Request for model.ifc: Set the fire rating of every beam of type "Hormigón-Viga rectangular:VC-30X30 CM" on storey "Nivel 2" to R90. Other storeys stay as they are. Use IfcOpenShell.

First a look at what the model holds.

```python
import ifcopenshell
import ifcopenshell.util.element

model = ifcopenshell.open("model.ifc")
print(model.schema)
storey = next(s for s in model.by_type("IfcBuildingStorey") if s.Name == "Nivel 2")
beams = [e for e in ifcopenshell.util.element.get_decomposition(storey) if e.is_a("IfcBeam")]
seen = {}
for e in beams:
    element_type = ifcopenshell.util.element.get_type(e)
    key = (element_type.Name if element_type != e and element_type else None, ifcopenshell.util.element.get_pset(e, "Pset_BeamCommon", "FireRating"))
    seen[key] = seen.get(key, 0) + 1
for (name, value), count in sorted(seen.items(), key=str):
    print(count, "x", name, "|", value)
```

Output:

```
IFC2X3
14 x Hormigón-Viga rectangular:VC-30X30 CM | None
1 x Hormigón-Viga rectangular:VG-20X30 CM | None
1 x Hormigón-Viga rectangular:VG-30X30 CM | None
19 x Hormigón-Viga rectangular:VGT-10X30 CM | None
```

```python
import ifcopenshell
import ifcopenshell.api.pset
import ifcopenshell.util.element

model = ifcopenshell.open("model.ifc")

storey = next(s for s in model.by_type("IfcBuildingStorey") if s.Name == "Nivel 2")
beams = [e for e in ifcopenshell.util.element.get_decomposition(storey) if e.is_a("IfcBeam")]

count = 0
for e in beams:
    element_type = ifcopenshell.util.element.get_type(e)
    if element_type in (None, e) or element_type.Name != "Hormigón-Viga rectangular:VC-30X30 CM":
        continue
    # add_pset returns the element's existing set when there is one.
    pset = ifcopenshell.api.pset.add_pset(model, product=e, name="Pset_BeamCommon")
    ifcopenshell.api.pset.edit_pset(model, pset=pset, properties={"FireRating": "R90"})
    count += 1

print(count, "beams updated")

model.write("model_v2.ifc")
```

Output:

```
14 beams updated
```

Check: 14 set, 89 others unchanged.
